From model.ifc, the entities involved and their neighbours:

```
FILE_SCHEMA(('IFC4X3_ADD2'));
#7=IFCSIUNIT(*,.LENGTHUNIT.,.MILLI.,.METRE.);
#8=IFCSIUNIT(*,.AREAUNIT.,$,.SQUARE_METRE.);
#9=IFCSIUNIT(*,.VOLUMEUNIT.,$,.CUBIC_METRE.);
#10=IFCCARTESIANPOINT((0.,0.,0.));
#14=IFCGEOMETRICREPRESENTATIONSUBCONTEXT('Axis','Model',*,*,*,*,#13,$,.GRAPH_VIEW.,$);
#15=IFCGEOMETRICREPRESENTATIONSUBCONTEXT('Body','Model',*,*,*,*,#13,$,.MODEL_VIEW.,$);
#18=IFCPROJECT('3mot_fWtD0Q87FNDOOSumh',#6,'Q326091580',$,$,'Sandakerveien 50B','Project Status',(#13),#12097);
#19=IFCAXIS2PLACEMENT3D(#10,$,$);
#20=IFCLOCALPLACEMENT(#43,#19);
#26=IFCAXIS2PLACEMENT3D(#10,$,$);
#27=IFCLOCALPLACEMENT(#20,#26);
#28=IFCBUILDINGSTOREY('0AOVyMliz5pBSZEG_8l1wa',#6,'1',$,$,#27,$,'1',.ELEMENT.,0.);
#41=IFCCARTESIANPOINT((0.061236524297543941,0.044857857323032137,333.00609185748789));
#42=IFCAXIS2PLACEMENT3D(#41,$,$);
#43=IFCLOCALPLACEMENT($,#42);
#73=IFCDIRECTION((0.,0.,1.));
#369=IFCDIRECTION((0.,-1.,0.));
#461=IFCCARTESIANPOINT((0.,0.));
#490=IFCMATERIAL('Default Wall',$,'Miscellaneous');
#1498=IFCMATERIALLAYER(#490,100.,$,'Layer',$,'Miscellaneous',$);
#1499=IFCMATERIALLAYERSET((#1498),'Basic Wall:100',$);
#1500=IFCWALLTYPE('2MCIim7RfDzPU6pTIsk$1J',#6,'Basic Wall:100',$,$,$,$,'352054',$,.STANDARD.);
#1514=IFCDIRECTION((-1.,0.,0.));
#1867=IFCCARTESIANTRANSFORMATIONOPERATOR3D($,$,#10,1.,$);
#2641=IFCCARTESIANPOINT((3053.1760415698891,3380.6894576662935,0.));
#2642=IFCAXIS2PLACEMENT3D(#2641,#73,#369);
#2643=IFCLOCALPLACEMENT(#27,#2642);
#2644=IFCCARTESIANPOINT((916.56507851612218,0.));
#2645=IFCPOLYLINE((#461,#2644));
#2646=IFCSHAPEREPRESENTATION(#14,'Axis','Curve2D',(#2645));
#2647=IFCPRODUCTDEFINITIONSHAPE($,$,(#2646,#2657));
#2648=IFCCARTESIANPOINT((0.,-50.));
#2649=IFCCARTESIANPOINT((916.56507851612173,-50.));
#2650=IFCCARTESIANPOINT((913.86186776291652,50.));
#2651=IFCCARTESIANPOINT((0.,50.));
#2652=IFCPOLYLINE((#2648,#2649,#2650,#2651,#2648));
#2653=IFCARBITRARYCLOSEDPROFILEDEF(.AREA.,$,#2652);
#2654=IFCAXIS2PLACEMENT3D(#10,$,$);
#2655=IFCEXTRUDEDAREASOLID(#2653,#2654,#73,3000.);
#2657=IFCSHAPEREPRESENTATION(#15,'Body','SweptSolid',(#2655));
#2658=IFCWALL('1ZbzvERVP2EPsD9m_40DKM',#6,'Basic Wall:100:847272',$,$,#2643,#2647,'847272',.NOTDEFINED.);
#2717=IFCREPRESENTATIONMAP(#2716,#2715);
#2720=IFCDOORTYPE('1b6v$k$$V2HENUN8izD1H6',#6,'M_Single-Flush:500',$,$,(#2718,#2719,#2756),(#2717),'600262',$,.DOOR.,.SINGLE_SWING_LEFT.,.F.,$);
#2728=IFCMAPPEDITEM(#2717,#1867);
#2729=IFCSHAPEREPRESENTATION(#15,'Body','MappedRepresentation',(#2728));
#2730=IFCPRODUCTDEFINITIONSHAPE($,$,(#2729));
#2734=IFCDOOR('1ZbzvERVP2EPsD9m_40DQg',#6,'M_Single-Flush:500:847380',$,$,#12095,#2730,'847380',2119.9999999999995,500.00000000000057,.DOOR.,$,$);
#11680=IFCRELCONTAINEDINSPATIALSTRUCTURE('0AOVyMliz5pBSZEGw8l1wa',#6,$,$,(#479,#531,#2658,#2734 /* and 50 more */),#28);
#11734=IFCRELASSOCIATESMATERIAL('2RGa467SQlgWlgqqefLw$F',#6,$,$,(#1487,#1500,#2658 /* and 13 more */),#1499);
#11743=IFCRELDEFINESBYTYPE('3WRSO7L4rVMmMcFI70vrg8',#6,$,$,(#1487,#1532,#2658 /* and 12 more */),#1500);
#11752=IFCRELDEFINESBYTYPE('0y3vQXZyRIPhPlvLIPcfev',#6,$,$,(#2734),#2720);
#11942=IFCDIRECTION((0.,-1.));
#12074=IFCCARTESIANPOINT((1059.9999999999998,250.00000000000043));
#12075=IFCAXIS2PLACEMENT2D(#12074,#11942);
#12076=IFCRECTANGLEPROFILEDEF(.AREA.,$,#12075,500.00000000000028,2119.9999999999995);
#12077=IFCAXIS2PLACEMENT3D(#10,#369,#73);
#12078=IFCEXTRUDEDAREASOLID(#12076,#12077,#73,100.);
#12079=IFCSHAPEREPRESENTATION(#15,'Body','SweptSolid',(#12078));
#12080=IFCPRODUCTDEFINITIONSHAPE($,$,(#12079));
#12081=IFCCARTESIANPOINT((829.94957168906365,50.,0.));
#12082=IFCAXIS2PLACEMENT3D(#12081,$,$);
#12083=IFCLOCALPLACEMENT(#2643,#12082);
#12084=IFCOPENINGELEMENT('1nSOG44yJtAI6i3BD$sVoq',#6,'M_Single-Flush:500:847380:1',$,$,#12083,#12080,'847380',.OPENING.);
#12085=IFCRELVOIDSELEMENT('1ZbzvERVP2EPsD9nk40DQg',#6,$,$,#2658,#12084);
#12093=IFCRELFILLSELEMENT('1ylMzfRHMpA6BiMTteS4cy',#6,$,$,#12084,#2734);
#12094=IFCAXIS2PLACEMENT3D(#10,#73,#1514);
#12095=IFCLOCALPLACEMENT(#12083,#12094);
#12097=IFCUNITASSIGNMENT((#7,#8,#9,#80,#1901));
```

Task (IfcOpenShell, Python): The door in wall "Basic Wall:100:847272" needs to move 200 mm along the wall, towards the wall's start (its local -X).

```python
import ifcopenshell
import ifcopenshell.api.geometry
import ifcopenshell.util.placement
import ifcopenshell.util.unit

model = ifcopenshell.open("model.ifc")
unit_scale = ifcopenshell.util.unit.calculate_unit_scale(model)

door = model.by_guid("1ZbzvERVP2EPsD9m_40DQg")
opening = door.FillsVoids[0].RelatingOpeningElement
wall = opening.VoidsElements[0].RelatingBuildingElement

wall_matrix = ifcopenshell.util.placement.get_local_placement(wall.ObjectPlacement)
shift = wall_matrix[:3, 0] * -0.2 / unit_scale
before = ifcopenshell.util.placement.get_local_placement(door.ObjectPlacement)[:3, 3].copy()

# The door is placed relative to its opening, so it follows when the opening moves.
matrix = ifcopenshell.util.placement.get_local_placement(opening.ObjectPlacement)
matrix[:3, 3] += shift
ifcopenshell.api.geometry.edit_object_placement(
    model, product=opening, matrix=matrix, is_si=False, should_transform_children=True
)

after = ifcopenshell.util.placement.get_local_placement(door.ObjectPlacement)[:3, 3]
print("door moved by", (after - before).round(3) + 0.0)

model.write("model_v2.ifc")
```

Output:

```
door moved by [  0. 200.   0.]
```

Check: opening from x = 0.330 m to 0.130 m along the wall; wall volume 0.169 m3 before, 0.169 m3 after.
